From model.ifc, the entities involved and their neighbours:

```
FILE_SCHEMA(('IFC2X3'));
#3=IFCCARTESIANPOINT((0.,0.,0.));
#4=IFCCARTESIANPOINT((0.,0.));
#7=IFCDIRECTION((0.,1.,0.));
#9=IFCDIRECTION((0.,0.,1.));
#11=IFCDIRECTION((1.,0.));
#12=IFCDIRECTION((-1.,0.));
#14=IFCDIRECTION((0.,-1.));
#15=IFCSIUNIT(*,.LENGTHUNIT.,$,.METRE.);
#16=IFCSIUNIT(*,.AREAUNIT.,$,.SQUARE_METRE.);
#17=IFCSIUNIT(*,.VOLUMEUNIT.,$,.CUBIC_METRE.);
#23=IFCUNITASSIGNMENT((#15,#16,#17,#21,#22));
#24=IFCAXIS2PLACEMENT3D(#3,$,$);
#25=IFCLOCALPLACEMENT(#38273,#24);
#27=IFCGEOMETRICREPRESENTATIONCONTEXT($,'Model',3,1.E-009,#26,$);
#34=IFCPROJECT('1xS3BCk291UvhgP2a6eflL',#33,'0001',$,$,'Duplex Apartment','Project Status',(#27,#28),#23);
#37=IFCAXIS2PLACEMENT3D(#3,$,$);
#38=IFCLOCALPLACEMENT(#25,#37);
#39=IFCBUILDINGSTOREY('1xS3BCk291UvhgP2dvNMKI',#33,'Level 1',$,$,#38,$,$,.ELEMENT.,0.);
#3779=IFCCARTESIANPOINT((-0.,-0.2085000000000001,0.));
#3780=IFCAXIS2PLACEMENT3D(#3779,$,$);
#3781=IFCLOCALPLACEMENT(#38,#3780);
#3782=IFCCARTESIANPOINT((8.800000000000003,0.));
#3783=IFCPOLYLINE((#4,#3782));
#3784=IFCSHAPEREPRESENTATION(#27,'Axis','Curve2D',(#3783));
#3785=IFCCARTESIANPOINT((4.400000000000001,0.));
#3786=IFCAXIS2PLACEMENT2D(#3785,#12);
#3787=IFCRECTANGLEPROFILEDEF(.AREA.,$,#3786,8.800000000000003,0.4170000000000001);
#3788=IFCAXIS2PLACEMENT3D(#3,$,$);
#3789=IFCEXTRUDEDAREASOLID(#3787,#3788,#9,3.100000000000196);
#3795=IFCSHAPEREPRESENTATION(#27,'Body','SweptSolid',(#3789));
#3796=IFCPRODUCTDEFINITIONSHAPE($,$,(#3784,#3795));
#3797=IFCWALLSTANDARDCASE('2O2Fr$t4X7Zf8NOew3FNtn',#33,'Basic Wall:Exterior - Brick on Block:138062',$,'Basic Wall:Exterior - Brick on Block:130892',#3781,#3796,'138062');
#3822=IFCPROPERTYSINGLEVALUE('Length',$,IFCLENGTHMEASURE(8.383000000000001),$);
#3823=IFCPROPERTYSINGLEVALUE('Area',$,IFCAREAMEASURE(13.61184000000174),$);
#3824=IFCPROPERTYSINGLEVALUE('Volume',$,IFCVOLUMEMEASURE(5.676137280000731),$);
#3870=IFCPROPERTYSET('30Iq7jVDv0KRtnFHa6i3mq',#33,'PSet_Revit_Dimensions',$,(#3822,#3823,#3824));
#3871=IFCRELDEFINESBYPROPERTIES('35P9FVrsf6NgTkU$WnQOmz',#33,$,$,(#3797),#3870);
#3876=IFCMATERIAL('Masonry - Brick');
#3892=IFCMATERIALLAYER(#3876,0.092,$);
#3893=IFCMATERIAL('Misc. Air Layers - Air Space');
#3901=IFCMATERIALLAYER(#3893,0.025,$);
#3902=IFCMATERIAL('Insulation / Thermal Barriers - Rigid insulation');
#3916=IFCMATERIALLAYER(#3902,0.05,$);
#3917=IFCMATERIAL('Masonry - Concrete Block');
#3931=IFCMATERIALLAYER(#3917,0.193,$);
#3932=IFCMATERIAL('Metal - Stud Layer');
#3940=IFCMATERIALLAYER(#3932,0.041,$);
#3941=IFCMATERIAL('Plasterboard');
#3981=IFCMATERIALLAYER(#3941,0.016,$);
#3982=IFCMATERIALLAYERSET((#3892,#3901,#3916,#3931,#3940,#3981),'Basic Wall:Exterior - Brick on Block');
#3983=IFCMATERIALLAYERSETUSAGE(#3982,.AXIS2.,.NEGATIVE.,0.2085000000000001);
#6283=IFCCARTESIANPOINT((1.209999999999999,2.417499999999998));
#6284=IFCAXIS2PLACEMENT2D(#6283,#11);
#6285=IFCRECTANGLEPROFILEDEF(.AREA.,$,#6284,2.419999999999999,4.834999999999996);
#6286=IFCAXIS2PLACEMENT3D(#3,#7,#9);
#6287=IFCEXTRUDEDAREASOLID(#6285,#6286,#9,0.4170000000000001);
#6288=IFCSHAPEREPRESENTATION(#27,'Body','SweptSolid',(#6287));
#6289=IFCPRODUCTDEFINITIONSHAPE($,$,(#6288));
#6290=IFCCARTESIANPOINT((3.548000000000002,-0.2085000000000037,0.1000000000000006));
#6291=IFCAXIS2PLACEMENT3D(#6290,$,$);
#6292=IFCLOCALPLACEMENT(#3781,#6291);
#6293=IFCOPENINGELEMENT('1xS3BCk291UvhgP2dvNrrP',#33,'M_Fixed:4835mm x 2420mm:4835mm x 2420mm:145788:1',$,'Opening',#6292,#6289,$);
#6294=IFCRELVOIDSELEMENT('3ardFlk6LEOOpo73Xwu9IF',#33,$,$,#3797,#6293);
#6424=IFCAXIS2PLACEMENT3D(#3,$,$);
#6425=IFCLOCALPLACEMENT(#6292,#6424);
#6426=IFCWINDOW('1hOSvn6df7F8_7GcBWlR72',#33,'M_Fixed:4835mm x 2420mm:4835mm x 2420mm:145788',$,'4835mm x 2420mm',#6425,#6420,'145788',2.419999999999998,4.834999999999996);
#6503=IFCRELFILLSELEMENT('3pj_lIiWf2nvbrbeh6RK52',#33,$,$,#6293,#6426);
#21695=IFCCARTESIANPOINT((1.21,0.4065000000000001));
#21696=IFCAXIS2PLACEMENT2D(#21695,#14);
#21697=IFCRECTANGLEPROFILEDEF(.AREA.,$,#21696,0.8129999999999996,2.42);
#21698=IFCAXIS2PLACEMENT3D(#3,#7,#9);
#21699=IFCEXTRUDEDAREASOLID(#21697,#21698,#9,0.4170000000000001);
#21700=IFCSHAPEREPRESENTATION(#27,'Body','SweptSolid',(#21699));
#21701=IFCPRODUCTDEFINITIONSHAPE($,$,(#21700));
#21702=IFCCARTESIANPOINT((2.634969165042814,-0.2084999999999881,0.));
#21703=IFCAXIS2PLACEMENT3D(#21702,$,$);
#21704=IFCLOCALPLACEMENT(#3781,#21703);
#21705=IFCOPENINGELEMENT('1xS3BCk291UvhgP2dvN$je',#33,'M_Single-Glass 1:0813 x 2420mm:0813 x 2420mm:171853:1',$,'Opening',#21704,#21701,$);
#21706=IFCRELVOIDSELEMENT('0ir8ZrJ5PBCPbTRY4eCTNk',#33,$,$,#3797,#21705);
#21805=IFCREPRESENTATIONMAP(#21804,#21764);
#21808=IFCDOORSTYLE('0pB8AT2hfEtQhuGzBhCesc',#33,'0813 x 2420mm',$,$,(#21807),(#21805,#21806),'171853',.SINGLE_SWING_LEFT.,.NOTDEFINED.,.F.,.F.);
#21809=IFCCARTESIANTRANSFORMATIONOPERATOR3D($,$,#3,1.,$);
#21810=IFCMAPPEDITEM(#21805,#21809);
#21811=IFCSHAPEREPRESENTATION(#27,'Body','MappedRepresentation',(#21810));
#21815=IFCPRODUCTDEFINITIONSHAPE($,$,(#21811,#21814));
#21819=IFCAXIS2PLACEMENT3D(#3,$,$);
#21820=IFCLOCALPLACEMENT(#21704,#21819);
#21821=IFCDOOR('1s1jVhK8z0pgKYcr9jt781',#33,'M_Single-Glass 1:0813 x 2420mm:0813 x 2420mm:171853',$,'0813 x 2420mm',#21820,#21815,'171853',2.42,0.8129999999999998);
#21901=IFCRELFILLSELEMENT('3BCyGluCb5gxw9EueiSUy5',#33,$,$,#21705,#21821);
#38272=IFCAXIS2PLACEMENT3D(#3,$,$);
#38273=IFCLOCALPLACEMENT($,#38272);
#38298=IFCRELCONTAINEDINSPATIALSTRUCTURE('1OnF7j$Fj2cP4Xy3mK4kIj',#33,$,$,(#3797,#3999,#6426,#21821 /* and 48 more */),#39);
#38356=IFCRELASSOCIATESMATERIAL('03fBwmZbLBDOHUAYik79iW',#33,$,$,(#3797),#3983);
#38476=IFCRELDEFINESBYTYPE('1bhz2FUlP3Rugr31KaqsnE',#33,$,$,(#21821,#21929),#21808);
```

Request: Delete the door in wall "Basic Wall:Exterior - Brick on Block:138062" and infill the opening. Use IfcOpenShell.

```python
import ifcopenshell
import ifcopenshell.api.feature
import ifcopenshell.api.pset
import ifcopenshell.api.root
import ifcopenshell.geom
import ifcopenshell.util.element
import ifcopenshell.util.shape
import ifcopenshell.util.unit

model = ifcopenshell.open("model.ifc")
area_scale = ifcopenshell.util.unit.calculate_unit_scale(model, "AREAUNIT")
volume_scale = ifcopenshell.util.unit.calculate_unit_scale(model, "VOLUMEUNIT")
settings = ifcopenshell.geom.settings()


def volume(element):
    """Net volume in cubic metres, openings subtracted."""
    shape = ifcopenshell.geom.create_shape(settings, element)
    return ifcopenshell.util.shape.get_volume(shape.geometry)


door = model.by_guid("1s1jVhK8z0pgKYcr9jt781")
opening = door.FillsVoids[0].RelatingOpeningElement
wall = opening.VoidsElements[0].RelatingBuildingElement
before = volume(wall)

ifcopenshell.api.root.remove_product(model, product=door)
ifcopenshell.api.feature.remove_feature(model, feature=opening)

after = volume(wall)
thickness = 0.417  # wall thickness in metres

# Update the wall's stored quantities.
pset = model.by_id(ifcopenshell.util.element.get_pset(wall, "PSet_Revit_Dimensions", should_inherit=False)["id"])
ifcopenshell.api.pset.edit_pset(model, pset=pset, properties={
    "Area": model.create_entity("IfcAreaMeasure", after / thickness / area_scale),
    "Volume": model.create_entity("IfcVolumeMeasure", after / volume_scale),
})

print(f"wall volume {before:.3f} -> {after:.3f} m3")

model.write("model_edited.ifc")
```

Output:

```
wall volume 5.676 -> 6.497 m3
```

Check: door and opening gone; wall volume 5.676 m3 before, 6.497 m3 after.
